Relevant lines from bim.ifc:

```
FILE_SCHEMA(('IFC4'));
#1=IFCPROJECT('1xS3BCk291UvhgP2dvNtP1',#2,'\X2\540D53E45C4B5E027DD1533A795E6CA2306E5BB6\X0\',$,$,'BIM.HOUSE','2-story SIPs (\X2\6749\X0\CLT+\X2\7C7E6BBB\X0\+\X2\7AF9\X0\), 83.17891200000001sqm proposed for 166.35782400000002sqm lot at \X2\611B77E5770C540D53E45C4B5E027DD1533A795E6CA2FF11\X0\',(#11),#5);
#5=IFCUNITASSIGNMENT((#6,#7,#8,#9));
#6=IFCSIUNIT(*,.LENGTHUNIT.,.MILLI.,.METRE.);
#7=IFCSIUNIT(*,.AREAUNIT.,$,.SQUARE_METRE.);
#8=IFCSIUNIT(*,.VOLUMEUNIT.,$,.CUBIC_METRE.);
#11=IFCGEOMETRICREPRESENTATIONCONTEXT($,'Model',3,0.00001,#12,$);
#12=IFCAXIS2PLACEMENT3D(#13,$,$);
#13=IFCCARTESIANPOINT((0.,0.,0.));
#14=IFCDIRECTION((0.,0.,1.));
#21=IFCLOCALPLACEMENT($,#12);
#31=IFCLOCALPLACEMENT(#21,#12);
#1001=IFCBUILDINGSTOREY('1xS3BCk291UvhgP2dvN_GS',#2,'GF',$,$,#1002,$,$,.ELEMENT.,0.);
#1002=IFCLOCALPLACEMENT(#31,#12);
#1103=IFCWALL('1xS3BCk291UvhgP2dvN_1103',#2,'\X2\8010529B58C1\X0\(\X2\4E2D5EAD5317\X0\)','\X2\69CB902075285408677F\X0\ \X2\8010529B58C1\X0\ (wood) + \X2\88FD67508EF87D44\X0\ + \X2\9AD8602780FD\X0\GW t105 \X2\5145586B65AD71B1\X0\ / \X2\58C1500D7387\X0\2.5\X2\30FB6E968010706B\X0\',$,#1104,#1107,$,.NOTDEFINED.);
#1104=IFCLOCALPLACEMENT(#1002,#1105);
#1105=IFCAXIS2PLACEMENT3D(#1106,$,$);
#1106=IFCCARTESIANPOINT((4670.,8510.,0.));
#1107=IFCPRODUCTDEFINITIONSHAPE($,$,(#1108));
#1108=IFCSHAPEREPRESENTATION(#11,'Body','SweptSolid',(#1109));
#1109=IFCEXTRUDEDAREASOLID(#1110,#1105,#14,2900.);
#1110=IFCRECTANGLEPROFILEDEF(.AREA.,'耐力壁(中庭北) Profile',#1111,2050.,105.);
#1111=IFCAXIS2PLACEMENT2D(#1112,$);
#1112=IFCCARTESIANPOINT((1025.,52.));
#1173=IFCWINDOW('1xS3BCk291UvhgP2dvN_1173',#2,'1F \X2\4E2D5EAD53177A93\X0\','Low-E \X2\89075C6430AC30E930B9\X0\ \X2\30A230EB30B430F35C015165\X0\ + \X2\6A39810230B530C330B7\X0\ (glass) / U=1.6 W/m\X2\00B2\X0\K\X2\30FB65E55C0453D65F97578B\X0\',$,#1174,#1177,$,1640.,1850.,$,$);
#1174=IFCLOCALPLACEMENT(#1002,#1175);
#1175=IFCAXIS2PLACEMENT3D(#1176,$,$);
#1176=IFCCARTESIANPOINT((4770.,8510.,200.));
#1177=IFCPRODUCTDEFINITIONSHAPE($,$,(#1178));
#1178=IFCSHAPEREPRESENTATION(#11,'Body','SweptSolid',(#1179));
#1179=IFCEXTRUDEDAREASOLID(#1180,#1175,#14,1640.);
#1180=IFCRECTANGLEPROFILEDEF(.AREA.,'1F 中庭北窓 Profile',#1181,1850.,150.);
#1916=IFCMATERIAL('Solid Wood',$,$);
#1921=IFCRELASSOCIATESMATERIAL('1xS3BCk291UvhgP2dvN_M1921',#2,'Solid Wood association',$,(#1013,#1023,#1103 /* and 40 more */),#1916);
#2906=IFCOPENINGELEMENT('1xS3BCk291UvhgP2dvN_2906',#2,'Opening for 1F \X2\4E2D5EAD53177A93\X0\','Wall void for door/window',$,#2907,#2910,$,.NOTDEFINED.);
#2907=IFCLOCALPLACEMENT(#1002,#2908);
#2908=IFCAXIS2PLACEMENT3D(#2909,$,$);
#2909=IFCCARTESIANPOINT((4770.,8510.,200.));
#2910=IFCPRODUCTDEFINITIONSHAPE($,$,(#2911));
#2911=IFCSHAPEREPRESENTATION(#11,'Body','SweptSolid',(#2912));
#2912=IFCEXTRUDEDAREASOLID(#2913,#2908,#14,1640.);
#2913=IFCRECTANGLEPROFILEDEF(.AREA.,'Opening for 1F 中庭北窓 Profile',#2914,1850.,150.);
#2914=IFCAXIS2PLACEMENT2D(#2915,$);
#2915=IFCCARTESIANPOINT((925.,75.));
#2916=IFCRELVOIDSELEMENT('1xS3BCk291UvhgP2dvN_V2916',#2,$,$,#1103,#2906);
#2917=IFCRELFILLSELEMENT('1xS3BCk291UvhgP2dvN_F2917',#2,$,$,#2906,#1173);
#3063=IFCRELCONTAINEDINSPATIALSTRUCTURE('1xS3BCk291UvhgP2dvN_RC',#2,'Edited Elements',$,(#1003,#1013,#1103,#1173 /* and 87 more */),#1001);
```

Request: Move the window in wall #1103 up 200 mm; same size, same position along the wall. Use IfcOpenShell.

```python
import numpy as np
import ifcopenshell
import ifcopenshell.api.geometry
import ifcopenshell.util.placement
import ifcopenshell.util.unit

model = ifcopenshell.open("bim.ifc")
unit_scale = ifcopenshell.util.unit.calculate_unit_scale(model)

window = model.by_id(1173)
opening = window.FillsVoids[0].RelatingOpeningElement
dz = 0.2 / unit_scale

shift = np.array([0.0, 0.0, dz])
# The window is not placed relative to its opening, so move both.
for product in (opening, window):
    matrix = ifcopenshell.util.placement.get_local_placement(product.ObjectPlacement)
    matrix[:3, 3] += shift
    ifcopenshell.api.geometry.edit_object_placement(model, product=product, matrix=matrix, is_si=False)

print(f"moved by {dz * unit_scale:+.3f} m")

model.write("bim_v2.ifc")
```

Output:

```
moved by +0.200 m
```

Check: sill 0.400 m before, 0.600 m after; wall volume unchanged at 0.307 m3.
